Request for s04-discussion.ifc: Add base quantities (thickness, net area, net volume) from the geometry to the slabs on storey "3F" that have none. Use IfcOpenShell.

First a look at what the model holds.

```python
import ifcopenshell
import ifcopenshell.util.element
import ifcopenshell.util.unit

model = ifcopenshell.open("s04-discussion.ifc")
print(model.schema)
for unit_type in ("LENGTHUNIT", "AREAUNIT", "VOLUMEUNIT"):
    print(unit_type, ifcopenshell.util.unit.calculate_unit_scale(model, unit_type))
storey = next(s for s in model.by_type("IfcBuildingStorey") if s.Name == "3F")
slabs = [e for e in ifcopenshell.util.element.get_decomposition(storey) if e.is_a("IfcSlab")]
for e in sorted(slabs, key=lambda e: e.id()):
    print(e.id(), e.is_a(), e.Name, list(ifcopenshell.util.element.get_psets(e, qtos_only=True)), sep=" | ")
```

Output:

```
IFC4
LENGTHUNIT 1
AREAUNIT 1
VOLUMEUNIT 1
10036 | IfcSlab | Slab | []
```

```python
import ifcopenshell
import ifcopenshell.api.pset
import ifcopenshell.geom
import ifcopenshell.util.element
import ifcopenshell.util.shape
import ifcopenshell.util.unit

model = ifcopenshell.open("s04-discussion.ifc")
unit_scale = ifcopenshell.util.unit.calculate_unit_scale(model)
area_scale = ifcopenshell.util.unit.calculate_unit_scale(model, "AREAUNIT")
volume_scale = ifcopenshell.util.unit.calculate_unit_scale(model, "VOLUMEUNIT")
settings = ifcopenshell.geom.settings()

storey = next(s for s in model.by_type("IfcBuildingStorey") if s.Name == "3F")
slabs = [e for e in ifcopenshell.util.element.get_decomposition(storey) if e.is_a("IfcSlab")]

for e in sorted(slabs, key=lambda e: e.id()):
    if ifcopenshell.util.element.get_psets(e, qtos_only=True, should_inherit=False):
        continue
    # Geometry comes back in metres, in the element's own axes.
    shape = ifcopenshell.geom.create_shape(settings, e)
    values = {
        "Width": ifcopenshell.util.shape.get_z(shape.geometry) / unit_scale,
        "NetArea": ifcopenshell.util.shape.get_footprint_area(shape.geometry) / area_scale,
        "NetVolume": ifcopenshell.util.shape.get_volume(shape.geometry) / volume_scale,
    }
    qto = ifcopenshell.api.pset.add_qto(model, product=e, name="Qto_SlabBaseQuantities")
    ifcopenshell.api.pset.edit_qto(model, qto=qto, properties=values)
    print(e.id(), {k: round(v, 3) for k, v in values.items()})

model.write("s04-discussion_rev.ifc")
```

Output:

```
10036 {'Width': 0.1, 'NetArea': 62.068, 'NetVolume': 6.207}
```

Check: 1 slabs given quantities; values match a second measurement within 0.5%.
